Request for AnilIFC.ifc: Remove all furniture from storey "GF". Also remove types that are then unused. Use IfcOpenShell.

First a look at what the model holds.

```python
import ifcopenshell
import ifcopenshell.util.element

model = ifcopenshell.open("AnilIFC.ifc")
print(model.schema)
storey = next(s for s in model.by_type("IfcBuildingStorey") if s.Name == "GF")
furniture = [e for e in ifcopenshell.util.element.get_decomposition(storey) if e.is_a("IfcFurnishingElement")]
seen = {}
for e in furniture:
    element_type = ifcopenshell.util.element.get_type(e)
    name = element_type.Name if element_type not in (None, e) else None
    seen[name] = seen.get(name, 0) + 1
for name, count in sorted(seen.items(), key=str):
    print(count, "x", name)
```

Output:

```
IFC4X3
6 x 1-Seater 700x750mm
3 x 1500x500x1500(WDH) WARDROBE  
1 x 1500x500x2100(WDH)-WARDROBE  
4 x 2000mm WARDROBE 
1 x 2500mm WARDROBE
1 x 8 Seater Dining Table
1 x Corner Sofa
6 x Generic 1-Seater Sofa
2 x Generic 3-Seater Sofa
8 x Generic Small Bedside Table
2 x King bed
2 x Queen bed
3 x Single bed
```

```python
import ifcopenshell
import ifcopenshell.api.root
import ifcopenshell.util.element

model = ifcopenshell.open("AnilIFC.ifc")

storey = next(s for s in model.by_type("IfcBuildingStorey") if s.Name == "GF")
furniture = [e for e in ifcopenshell.util.element.get_decomposition(storey) if e.is_a("IfcFurnishingElement")]
types = {ifcopenshell.util.element.get_type(e) for e in furniture} - {None, *furniture}

for e in furniture:
    ifcopenshell.api.root.remove_product(model, product=e)
print(len(furniture), "removed")

unused = [t for t in types if not ifcopenshell.util.element.get_types(t)]
for t in unused:
    ifcopenshell.api.root.remove_product(model, product=t)
print(len(unused), "unused types removed")

model.write("AnilIFC-out.ifc")
```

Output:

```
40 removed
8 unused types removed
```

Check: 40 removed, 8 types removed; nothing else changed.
